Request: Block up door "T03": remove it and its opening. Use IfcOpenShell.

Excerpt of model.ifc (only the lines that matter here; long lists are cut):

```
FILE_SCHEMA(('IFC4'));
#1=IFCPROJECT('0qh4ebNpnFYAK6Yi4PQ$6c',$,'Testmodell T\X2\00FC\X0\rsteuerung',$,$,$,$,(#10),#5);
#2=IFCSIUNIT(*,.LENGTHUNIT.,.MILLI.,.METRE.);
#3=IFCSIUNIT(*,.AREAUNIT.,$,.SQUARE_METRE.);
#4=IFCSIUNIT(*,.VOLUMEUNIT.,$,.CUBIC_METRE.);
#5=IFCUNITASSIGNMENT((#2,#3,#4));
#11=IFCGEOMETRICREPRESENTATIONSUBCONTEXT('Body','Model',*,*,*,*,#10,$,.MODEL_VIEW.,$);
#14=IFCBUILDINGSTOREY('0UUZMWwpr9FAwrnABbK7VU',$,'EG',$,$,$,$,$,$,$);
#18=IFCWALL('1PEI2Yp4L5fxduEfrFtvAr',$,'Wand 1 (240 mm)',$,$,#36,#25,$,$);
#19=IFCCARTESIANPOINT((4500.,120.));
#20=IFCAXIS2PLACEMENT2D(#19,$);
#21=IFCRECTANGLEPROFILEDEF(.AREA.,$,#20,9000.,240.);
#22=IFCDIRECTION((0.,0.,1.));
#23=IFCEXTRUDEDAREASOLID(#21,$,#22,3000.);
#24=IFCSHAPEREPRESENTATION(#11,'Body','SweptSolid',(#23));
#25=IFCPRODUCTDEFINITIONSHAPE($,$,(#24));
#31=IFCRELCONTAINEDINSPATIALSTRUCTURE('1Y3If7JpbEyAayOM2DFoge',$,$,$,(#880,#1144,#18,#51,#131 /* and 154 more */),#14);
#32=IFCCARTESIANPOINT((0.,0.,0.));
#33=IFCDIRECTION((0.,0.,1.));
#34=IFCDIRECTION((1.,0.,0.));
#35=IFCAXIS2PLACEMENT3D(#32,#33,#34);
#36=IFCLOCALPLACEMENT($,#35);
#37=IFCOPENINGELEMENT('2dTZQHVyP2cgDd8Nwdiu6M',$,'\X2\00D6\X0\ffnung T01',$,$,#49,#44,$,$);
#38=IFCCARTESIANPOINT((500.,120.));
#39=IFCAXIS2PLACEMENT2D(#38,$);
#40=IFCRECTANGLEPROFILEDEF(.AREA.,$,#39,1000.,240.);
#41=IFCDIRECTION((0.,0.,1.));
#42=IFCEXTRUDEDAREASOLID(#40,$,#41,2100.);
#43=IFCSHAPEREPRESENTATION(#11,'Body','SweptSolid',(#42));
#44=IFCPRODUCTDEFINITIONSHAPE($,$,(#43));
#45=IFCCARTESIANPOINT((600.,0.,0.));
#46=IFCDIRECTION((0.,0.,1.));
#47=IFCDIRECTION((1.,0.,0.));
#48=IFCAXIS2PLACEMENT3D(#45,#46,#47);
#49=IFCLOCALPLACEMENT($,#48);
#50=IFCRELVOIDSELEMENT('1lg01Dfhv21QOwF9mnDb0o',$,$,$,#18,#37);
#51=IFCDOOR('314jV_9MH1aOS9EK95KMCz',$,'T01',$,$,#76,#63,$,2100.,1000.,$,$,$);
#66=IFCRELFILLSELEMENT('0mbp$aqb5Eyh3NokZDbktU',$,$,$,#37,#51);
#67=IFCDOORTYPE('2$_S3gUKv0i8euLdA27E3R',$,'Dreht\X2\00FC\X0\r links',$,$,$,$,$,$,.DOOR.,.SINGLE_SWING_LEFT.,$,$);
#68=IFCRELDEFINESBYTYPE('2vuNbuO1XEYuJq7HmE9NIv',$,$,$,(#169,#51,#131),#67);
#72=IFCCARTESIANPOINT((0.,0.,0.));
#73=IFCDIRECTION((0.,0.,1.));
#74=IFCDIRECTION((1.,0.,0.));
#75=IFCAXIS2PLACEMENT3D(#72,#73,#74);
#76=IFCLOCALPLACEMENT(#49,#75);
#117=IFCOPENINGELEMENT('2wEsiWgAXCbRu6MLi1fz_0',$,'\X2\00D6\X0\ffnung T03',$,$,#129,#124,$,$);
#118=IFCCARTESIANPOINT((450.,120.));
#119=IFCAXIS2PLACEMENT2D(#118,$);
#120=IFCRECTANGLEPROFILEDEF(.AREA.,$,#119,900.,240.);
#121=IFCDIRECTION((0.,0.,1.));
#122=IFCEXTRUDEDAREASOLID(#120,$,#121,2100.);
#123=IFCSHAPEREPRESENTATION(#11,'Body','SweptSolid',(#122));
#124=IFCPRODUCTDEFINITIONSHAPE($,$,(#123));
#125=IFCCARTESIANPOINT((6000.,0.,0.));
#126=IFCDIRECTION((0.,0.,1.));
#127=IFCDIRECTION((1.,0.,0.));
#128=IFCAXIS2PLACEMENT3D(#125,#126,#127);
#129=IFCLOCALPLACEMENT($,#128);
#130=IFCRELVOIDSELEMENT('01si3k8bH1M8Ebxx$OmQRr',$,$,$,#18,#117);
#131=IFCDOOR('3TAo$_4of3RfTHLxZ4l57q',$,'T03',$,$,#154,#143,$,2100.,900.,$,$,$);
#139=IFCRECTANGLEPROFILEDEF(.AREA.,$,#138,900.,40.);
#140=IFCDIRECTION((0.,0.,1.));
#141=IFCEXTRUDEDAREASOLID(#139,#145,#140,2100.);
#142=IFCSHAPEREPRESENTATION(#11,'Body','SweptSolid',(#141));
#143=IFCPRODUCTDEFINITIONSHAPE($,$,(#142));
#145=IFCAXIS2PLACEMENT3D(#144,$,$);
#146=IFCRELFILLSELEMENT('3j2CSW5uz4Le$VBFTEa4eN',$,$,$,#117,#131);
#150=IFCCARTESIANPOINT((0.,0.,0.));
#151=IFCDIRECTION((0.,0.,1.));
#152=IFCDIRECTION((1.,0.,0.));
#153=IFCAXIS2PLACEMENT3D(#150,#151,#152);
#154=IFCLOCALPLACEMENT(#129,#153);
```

```python
import ifcopenshell
import ifcopenshell.api.feature
import ifcopenshell.api.root
import ifcopenshell.geom
import ifcopenshell.util.shape

model = ifcopenshell.open("model.ifc")
settings = ifcopenshell.geom.settings()


def volume(element):
    """Net volume in cubic metres, openings subtracted."""
    shape = ifcopenshell.geom.create_shape(settings, element)
    return ifcopenshell.util.shape.get_volume(shape.geometry)


door = model.by_guid("3TAo$_4of3RfTHLxZ4l57q")
opening = door.FillsVoids[0].RelatingOpeningElement
wall = opening.VoidsElements[0].RelatingBuildingElement
before = volume(wall)

ifcopenshell.api.root.remove_product(model, product=door)
ifcopenshell.api.feature.remove_feature(model, feature=opening)

after = volume(wall)

print(f"wall volume {before:.3f} -> {after:.3f} m3")

model.write("model_updated.ifc")
```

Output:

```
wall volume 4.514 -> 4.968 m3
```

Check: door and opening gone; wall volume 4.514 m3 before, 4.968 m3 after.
